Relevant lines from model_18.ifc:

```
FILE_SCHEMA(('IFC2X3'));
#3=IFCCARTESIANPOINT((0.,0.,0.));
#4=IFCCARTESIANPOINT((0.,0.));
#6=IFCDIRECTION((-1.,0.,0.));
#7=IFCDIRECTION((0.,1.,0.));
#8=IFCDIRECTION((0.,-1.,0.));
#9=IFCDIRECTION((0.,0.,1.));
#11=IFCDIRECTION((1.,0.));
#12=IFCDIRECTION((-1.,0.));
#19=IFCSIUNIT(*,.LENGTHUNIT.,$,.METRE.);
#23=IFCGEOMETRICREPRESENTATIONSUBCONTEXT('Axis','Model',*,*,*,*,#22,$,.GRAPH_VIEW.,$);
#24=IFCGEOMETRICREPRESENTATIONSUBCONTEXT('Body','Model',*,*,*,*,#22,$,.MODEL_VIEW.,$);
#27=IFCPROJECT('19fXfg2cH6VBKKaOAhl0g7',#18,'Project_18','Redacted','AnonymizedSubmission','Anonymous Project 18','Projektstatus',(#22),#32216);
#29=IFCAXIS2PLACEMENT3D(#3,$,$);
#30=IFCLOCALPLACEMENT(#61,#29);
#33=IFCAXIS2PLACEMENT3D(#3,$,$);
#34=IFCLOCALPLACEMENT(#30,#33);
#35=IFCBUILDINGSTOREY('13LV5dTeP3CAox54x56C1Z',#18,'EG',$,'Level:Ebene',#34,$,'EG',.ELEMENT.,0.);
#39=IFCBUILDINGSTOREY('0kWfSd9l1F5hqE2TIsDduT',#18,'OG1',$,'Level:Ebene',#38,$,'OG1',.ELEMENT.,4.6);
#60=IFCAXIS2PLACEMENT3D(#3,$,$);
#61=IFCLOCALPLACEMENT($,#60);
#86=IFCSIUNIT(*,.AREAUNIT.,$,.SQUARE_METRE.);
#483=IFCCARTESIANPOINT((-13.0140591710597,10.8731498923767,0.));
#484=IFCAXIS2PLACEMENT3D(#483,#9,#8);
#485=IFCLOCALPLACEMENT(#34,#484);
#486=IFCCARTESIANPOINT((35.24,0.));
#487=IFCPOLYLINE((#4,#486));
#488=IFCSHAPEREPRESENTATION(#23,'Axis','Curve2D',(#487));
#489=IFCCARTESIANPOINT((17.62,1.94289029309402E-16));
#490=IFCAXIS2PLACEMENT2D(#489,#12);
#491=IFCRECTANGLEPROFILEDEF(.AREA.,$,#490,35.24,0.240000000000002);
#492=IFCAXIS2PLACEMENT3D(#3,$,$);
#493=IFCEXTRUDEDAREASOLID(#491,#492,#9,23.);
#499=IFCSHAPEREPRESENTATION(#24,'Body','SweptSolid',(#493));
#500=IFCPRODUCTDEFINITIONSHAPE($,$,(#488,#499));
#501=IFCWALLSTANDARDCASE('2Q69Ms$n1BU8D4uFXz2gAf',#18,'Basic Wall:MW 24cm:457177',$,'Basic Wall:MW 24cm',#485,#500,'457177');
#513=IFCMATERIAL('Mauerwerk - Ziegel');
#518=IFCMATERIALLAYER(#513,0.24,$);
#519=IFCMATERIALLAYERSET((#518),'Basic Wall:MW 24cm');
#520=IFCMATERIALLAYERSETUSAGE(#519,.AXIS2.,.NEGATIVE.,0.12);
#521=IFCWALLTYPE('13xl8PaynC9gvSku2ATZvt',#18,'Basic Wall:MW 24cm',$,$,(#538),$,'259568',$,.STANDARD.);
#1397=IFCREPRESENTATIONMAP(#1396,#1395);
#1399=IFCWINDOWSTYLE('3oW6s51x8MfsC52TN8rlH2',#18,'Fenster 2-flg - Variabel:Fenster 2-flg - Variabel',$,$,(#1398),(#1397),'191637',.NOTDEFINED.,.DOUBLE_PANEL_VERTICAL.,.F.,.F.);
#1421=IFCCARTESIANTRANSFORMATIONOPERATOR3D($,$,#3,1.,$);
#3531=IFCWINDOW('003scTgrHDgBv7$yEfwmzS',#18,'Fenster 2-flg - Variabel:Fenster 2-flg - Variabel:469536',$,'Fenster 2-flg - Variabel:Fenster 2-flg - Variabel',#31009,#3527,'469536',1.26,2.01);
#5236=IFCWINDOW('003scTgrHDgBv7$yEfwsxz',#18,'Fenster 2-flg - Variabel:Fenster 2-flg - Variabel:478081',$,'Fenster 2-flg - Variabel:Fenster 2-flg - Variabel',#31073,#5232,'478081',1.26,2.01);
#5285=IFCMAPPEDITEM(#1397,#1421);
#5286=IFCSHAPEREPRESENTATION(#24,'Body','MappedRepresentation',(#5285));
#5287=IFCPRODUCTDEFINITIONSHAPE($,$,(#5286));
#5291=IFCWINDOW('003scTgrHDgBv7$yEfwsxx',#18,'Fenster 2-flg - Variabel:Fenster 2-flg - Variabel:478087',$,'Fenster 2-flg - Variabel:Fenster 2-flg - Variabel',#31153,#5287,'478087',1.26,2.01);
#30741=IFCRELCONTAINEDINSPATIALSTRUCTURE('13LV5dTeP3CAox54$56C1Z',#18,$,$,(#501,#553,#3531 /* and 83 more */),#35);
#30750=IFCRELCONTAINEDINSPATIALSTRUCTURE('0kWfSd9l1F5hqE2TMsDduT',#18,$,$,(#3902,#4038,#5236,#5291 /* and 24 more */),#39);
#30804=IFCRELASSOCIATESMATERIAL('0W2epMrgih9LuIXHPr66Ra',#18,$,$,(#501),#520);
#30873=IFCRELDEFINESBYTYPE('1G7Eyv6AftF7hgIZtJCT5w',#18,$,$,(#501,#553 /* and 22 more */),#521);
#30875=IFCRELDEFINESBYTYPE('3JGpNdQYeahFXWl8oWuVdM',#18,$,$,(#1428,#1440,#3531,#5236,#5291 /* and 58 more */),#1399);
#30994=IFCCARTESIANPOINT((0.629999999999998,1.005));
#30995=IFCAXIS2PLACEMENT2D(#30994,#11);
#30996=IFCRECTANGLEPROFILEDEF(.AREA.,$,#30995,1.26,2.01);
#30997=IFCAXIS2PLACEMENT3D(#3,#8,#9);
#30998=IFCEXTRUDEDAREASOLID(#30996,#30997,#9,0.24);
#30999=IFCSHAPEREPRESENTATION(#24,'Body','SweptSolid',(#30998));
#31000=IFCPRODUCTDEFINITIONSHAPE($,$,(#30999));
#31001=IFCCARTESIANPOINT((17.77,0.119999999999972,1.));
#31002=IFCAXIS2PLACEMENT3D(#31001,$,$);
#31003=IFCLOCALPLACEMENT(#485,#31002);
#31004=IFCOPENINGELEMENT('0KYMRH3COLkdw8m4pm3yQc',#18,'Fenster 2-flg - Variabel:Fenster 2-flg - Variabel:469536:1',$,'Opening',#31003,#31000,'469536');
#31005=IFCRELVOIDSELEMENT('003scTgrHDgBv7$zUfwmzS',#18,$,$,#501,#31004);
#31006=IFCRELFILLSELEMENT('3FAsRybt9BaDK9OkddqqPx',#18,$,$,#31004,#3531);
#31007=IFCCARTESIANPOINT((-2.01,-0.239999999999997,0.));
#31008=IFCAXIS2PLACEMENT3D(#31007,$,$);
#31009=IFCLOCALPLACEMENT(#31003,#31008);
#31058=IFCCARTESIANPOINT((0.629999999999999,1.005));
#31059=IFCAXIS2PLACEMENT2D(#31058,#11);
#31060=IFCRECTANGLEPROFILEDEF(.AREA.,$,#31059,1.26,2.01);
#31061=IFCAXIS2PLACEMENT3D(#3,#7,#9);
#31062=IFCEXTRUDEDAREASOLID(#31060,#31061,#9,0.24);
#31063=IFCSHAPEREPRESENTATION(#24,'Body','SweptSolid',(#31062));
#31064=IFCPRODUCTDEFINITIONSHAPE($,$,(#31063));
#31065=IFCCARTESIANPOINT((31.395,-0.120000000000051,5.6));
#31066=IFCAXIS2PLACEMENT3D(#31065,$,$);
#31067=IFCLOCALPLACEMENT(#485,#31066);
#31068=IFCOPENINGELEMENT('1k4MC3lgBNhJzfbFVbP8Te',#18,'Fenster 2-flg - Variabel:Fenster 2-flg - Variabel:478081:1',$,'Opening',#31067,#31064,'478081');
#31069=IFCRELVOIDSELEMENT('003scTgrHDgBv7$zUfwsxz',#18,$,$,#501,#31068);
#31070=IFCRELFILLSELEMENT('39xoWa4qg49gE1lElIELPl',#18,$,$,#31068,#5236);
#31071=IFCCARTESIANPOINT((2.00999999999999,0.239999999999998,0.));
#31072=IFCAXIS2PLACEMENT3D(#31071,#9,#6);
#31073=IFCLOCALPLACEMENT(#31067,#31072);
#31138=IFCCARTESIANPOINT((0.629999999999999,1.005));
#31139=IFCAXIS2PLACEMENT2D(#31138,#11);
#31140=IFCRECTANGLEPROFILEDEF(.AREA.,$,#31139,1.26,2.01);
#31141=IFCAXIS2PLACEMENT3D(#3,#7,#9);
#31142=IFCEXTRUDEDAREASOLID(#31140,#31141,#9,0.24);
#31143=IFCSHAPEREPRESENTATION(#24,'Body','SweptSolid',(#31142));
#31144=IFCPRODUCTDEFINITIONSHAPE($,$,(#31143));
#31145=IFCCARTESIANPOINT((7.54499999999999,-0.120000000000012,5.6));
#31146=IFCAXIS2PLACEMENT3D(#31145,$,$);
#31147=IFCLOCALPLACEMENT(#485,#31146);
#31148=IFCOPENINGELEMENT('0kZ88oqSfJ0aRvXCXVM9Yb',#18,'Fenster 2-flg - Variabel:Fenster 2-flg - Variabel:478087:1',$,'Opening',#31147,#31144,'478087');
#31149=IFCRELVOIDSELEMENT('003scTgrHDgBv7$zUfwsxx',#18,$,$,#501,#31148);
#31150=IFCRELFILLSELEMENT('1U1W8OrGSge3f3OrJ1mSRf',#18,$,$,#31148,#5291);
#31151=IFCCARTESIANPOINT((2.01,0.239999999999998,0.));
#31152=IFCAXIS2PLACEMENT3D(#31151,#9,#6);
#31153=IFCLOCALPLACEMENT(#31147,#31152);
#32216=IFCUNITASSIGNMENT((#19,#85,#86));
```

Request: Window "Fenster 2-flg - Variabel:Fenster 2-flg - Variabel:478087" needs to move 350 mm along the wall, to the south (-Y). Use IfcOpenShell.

```python
import ifcopenshell
import ifcopenshell.api.geometry
import ifcopenshell.util.placement
import ifcopenshell.util.unit

model = ifcopenshell.open("model_18.ifc")
unit_scale = ifcopenshell.util.unit.calculate_unit_scale(model)

window = model.by_guid("003scTgrHDgBv7$yEfwsxx")
opening = window.FillsVoids[0].RelatingOpeningElement
wall = opening.VoidsElements[0].RelatingBuildingElement

wall_matrix = ifcopenshell.util.placement.get_local_placement(wall.ObjectPlacement)
shift = wall_matrix[:3, 0] * 0.35 / unit_scale
before = ifcopenshell.util.placement.get_local_placement(window.ObjectPlacement)[:3, 3].copy()

# The window is placed relative to its opening, so it follows when the opening moves.
matrix = ifcopenshell.util.placement.get_local_placement(opening.ObjectPlacement)
matrix[:3, 3] += shift
ifcopenshell.api.geometry.edit_object_placement(
    model, product=opening, matrix=matrix, is_si=False, should_transform_children=True
)

after = ifcopenshell.util.placement.get_local_placement(window.ObjectPlacement)[:3, 3]
print("window moved by", (after - before).round(3) + 0.0)

model.write("model_18_edited.ifc")
```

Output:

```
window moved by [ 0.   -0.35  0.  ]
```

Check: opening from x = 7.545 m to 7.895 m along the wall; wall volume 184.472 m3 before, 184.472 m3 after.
